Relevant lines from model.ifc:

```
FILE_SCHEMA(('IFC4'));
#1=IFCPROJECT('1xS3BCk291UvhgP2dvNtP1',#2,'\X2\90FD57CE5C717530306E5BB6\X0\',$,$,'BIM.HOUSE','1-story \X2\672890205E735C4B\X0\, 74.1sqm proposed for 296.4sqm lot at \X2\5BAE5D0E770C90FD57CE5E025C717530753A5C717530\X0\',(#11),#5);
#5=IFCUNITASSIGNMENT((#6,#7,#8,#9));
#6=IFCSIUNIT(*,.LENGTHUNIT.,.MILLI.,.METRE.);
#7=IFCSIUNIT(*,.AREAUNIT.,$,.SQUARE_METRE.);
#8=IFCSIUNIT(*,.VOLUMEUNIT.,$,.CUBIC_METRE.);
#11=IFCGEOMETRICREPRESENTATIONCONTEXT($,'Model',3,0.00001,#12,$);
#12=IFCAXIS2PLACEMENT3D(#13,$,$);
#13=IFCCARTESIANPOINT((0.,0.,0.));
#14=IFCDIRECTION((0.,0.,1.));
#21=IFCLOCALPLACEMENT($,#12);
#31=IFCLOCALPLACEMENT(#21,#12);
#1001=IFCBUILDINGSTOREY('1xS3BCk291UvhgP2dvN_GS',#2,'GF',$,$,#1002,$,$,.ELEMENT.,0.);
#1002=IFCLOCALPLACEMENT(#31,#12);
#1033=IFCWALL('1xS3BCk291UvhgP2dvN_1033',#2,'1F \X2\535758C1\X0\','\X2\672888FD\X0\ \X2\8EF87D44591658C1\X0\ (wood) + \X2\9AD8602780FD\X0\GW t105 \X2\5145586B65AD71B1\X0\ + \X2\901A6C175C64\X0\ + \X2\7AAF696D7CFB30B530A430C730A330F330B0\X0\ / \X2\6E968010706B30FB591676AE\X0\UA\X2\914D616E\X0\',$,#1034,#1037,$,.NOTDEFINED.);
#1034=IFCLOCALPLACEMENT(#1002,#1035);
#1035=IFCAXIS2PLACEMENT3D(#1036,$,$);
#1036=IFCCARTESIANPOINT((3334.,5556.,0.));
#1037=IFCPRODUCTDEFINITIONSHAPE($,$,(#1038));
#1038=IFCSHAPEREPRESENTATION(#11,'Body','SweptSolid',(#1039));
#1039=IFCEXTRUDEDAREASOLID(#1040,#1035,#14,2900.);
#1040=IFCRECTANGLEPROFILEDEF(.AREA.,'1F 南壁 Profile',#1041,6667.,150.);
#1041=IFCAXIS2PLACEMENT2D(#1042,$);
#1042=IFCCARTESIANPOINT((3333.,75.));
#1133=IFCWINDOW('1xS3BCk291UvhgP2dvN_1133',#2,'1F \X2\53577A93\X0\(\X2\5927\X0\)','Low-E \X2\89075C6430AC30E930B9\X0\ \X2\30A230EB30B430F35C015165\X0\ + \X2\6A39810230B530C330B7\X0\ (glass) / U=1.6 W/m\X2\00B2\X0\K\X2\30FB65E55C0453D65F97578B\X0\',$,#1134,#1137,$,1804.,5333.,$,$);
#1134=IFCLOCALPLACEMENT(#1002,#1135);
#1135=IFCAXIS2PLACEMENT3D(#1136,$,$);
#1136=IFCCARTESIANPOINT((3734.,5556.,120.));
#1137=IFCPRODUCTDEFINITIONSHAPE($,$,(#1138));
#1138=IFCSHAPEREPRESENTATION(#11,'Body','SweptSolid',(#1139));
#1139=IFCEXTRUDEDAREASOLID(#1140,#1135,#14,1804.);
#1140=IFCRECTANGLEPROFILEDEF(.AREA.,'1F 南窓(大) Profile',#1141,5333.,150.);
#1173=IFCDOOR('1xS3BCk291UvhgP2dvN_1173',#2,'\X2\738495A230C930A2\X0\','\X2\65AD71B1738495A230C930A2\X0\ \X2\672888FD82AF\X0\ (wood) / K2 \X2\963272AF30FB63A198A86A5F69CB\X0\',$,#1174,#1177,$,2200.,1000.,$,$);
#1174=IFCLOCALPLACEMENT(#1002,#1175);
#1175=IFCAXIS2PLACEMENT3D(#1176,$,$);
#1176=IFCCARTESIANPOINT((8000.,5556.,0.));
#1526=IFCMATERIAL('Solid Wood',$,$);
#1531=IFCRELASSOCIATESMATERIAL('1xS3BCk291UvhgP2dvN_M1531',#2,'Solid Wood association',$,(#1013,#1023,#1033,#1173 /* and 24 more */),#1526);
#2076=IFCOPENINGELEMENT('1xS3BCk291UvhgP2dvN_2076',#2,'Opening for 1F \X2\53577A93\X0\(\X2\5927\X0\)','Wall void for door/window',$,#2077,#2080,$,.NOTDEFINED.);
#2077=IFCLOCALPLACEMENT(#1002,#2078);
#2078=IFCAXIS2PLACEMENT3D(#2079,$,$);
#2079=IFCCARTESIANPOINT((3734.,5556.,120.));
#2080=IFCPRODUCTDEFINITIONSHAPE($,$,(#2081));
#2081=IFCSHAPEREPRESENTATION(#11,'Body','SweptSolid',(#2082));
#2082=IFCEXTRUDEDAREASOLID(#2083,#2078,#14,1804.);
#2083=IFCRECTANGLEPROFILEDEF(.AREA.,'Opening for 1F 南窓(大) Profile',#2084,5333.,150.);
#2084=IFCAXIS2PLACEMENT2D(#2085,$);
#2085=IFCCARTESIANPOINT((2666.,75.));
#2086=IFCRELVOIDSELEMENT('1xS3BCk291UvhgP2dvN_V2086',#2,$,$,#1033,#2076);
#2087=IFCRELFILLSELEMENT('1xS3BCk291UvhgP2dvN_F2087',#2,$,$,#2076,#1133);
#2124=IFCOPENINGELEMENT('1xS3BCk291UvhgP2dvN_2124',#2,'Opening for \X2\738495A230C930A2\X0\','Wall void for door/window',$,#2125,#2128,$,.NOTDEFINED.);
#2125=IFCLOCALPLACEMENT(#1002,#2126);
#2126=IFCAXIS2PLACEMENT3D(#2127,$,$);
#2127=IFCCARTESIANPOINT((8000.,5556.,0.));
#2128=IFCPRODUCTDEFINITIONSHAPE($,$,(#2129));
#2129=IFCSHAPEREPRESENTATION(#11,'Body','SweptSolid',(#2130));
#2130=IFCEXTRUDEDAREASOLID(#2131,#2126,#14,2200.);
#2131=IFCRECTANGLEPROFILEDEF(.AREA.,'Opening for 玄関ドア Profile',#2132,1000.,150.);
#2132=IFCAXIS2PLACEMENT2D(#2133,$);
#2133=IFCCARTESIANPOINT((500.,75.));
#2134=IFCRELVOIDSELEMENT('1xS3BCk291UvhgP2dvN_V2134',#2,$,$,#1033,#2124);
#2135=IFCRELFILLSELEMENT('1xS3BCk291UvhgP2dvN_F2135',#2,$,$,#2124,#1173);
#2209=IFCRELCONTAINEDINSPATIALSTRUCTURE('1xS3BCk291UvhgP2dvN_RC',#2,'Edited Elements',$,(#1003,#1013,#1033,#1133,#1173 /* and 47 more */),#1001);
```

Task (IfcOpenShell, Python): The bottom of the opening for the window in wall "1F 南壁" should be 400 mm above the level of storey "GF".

```python
import numpy as np
import ifcopenshell
import ifcopenshell.api.geometry
import ifcopenshell.geom
import ifcopenshell.util.element
import ifcopenshell.util.placement
import ifcopenshell.util.shape
import ifcopenshell.util.unit

model = ifcopenshell.open("model.ifc")
unit_scale = ifcopenshell.util.unit.calculate_unit_scale(model)

window = model.by_id(1133)
opening = window.FillsVoids[0].RelatingOpeningElement
storey = ifcopenshell.util.element.get_container(window, ifc_class="IfcBuildingStorey")
level = ifcopenshell.util.placement.get_local_placement(storey.ObjectPlacement)[2, 3]

# The opening's origin need not be at the sill, so measure its lowest point.
shape = ifcopenshell.geom.create_shape(ifcopenshell.geom.settings(), opening)
bottom = ifcopenshell.util.shape.get_shape_bottom_elevation(shape, shape.geometry) / unit_scale
dz = level + 0.4 / unit_scale - bottom

shift = np.array([0.0, 0.0, dz])
# The window is not placed relative to its opening, so move both.
for product in (opening, window):
    matrix = ifcopenshell.util.placement.get_local_placement(product.ObjectPlacement)
    matrix[:3, 3] += shift
    ifcopenshell.api.geometry.edit_object_placement(model, product=product, matrix=matrix, is_si=False)

print(f"moved by {dz * unit_scale:+.3f} m")

model.write("model_updated.ifc")
```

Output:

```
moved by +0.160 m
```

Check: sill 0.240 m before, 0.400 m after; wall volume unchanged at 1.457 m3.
